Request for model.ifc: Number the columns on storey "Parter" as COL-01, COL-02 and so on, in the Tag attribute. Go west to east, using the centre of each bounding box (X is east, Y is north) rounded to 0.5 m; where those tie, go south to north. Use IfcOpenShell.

First a look at what the model holds.

```python
import ifcopenshell
import ifcopenshell.util.element
import ifcopenshell.util.placement

model = ifcopenshell.open("model.ifc")
print(model.schema)
storey = next(s for s in model.by_type("IfcBuildingStorey") if s.Name == "Parter")
columns = [e for e in ifcopenshell.util.element.get_decomposition(storey) if e.is_a("IfcColumn")]
for e in sorted(columns, key=lambda e: e.id()):
    origin = ifcopenshell.util.placement.get_local_placement(e.ObjectPlacement)[:3, 3]
    print(e.id(), e.Tag, e.Name, origin.round(2) + 0.0, sep=" | ")
```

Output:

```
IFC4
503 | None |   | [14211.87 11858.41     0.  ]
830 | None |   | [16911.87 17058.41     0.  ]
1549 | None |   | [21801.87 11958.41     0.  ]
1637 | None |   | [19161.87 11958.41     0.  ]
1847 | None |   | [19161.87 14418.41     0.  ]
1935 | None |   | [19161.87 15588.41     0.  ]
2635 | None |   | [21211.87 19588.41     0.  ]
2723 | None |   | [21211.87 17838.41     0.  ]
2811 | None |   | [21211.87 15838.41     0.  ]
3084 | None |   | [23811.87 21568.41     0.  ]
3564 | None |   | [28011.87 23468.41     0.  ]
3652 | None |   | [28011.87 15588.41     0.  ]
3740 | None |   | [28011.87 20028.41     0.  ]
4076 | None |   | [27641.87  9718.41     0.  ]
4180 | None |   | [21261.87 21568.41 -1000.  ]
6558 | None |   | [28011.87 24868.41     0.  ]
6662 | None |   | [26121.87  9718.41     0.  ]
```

```python
import ifcopenshell
import ifcopenshell.geom
import ifcopenshell.util.element
import ifcopenshell.util.shape

model = ifcopenshell.open("model.ifc")
settings = ifcopenshell.geom.settings()
settings.set("use-world-coords", True)


def centre(element):
    shape = ifcopenshell.geom.create_shape(settings, element)
    return ifcopenshell.util.shape.get_bbox_centroid(shape.geometry)


storey = next(s for s in model.by_type("IfcBuildingStorey") if s.Name == "Parter")
columns = [e for e in ifcopenshell.util.element.get_decomposition(storey) if e.is_a("IfcColumn")]

# Insertion points can sit at a corner or the storey origin, so sort by the geometry (in metres).
centres = {e: centre(e) for e in columns}
columns.sort(key=lambda e: (round(centres[e][0] / 0.5), centres[e][1]))

for i, e in enumerate(columns, start=1):
    number = f"COL-{i:02d}"
    e.Tag = number
    print(e.id(), number)

model.write("model_v2.ifc")
```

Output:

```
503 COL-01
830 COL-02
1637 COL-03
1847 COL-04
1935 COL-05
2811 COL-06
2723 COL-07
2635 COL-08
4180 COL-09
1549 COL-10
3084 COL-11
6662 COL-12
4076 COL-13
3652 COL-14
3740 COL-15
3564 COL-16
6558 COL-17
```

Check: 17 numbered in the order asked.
